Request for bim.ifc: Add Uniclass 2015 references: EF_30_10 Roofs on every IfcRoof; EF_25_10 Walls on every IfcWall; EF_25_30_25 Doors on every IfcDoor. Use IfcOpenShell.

First a look at what the model holds.

```python
import ifcopenshell

model = ifcopenshell.open("bim.ifc")
print(model.schema)
print("classifications:", [c.Name for c in model.by_type("IfcClassification")])
for ifc_class in ("IfcDoor", "IfcRoof", "IfcStair", "IfcWall", "IfcWindow"):
    print(ifc_class, len(model.by_type(ifc_class)))
```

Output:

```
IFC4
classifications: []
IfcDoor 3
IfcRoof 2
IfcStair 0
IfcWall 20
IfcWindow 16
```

```python
import ifcopenshell
import ifcopenshell.api.classification

model = ifcopenshell.open("bim.ifc")

system = ifcopenshell.api.classification.add_classification(model, classification="Uniclass 2015")

codes = {
    "IfcRoof": ("EF_30_10", "Roofs"),
    "IfcWall": ("EF_25_10", "Walls"),
    "IfcDoor": ("EF_25_30_25", "Doors"),
}
for ifc_class, (code, name) in codes.items():
    products = model.by_type(ifc_class)
    ifcopenshell.api.classification.add_reference(
        model, products=products, classification=system, identification=code, name=name
    )
    print(code, len(products))

model.write("bim_edited.ifc")
```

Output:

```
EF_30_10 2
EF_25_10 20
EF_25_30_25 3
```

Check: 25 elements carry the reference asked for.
